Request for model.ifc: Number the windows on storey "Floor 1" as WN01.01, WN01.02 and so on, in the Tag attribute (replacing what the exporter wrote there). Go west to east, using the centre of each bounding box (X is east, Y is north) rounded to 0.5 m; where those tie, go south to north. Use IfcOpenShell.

First a look at what the model holds.

```python
import ifcopenshell
import ifcopenshell.util.element
import ifcopenshell.util.placement

model = ifcopenshell.open("model.ifc")
print(model.schema)
storey = next(s for s in model.by_type("IfcBuildingStorey") if s.Name == "Floor 1")
windows = [e for e in ifcopenshell.util.element.get_decomposition(storey) if e.is_a("IfcWindow")]
for e in sorted(windows, key=lambda e: e.id()):
    origin = ifcopenshell.util.placement.get_local_placement(e.ObjectPlacement)[:3, 3]
    print(e.id(), e.Tag, e.Name, origin.round(2) + 0.0, sep=" | ")
```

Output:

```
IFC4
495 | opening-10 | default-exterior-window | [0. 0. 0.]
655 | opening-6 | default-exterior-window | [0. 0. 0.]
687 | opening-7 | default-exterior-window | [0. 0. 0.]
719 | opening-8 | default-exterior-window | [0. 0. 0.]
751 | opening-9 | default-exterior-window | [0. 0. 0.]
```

```python
import ifcopenshell
import ifcopenshell.geom
import ifcopenshell.util.element
import ifcopenshell.util.shape

model = ifcopenshell.open("model.ifc")
settings = ifcopenshell.geom.settings()
settings.set("use-world-coords", True)


def centre(element):
    shape = ifcopenshell.geom.create_shape(settings, element)
    return ifcopenshell.util.shape.get_bbox_centroid(shape.geometry)


storey = next(s for s in model.by_type("IfcBuildingStorey") if s.Name == "Floor 1")
windows = [e for e in ifcopenshell.util.element.get_decomposition(storey) if e.is_a("IfcWindow")]

# Insertion points can sit at a corner or the storey origin, so sort by the geometry (in metres).
centres = {e: centre(e) for e in windows}
windows.sort(key=lambda e: (round(centres[e][0] / 0.5), centres[e][1]))

for i, e in enumerate(windows, start=1):
    number = f"WN01.{i:02d}"
    e.Tag = number
    print(e.id(), number)

model.write("model_updated.ifc")
```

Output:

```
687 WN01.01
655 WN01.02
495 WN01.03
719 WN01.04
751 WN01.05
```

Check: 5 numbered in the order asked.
